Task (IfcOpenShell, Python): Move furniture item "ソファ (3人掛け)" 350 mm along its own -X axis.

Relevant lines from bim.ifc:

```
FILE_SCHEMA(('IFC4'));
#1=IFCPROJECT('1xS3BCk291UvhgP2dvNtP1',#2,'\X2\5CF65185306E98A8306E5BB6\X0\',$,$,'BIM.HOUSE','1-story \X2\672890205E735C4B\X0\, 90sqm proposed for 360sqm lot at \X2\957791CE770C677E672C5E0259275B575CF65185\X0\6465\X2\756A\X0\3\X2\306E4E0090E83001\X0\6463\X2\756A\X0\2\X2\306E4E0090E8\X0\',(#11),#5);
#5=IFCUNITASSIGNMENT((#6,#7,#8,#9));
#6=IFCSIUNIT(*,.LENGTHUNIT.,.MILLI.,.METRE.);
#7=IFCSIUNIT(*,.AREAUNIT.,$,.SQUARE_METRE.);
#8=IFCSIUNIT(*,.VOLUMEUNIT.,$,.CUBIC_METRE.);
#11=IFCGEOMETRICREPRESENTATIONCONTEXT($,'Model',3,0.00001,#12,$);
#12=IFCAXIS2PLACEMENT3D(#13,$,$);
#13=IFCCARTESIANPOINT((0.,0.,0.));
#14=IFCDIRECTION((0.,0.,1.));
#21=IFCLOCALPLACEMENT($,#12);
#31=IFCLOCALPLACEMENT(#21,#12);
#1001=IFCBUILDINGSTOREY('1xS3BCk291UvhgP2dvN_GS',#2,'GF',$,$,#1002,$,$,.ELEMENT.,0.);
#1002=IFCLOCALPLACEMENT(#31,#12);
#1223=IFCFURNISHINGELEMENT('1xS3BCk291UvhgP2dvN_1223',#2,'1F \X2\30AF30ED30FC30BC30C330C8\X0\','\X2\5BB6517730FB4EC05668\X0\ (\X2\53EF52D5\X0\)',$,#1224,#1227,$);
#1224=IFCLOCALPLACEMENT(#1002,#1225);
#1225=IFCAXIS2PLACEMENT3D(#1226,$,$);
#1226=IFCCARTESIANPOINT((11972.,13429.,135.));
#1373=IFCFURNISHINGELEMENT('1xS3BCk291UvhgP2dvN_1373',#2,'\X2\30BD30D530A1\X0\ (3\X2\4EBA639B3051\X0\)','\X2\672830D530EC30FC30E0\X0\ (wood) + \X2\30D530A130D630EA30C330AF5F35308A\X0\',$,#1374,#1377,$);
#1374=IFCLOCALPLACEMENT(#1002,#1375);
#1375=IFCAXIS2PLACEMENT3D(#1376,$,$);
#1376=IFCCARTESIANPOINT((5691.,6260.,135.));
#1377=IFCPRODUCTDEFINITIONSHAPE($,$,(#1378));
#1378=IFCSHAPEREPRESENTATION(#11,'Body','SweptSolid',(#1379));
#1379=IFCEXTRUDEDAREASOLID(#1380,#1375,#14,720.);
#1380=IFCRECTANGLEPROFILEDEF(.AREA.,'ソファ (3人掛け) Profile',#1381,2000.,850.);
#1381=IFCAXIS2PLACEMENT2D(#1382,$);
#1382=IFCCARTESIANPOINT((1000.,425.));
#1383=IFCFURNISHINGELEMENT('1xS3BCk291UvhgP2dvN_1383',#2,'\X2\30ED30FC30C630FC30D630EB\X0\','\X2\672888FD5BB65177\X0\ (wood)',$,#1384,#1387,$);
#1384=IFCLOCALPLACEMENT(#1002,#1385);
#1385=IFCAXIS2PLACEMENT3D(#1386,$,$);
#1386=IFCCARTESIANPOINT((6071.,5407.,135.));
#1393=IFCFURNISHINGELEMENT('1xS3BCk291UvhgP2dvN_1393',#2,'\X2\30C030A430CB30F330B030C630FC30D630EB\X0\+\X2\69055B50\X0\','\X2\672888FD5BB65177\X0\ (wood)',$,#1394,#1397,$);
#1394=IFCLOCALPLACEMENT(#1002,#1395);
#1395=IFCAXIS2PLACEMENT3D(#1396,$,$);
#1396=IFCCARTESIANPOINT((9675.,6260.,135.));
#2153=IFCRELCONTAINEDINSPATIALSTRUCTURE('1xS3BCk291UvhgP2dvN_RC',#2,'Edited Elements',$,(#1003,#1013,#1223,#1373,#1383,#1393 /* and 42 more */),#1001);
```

```python
import ifcopenshell
import ifcopenshell.api.geometry
import ifcopenshell.util.placement
import ifcopenshell.util.unit

model = ifcopenshell.open("bim.ifc")
unit_scale = ifcopenshell.util.unit.calculate_unit_scale(model)

item = model.by_guid("1xS3BCk291UvhgP2dvN_1373")
matrix = ifcopenshell.util.placement.get_local_placement(item.ObjectPlacement)
matrix[:3, 3] -= matrix[:3, 0] * 0.35 / unit_scale
ifcopenshell.api.geometry.edit_object_placement(model, product=item, matrix=matrix, is_si=False)

print(ifcopenshell.util.placement.get_local_placement(item.ObjectPlacement).round(3) + 0.0)

model.write("bim_v2.ifc")
```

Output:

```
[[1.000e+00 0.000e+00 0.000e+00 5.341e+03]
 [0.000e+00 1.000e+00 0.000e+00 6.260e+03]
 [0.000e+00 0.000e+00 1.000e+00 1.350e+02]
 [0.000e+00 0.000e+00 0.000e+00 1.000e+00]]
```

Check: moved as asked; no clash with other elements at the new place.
